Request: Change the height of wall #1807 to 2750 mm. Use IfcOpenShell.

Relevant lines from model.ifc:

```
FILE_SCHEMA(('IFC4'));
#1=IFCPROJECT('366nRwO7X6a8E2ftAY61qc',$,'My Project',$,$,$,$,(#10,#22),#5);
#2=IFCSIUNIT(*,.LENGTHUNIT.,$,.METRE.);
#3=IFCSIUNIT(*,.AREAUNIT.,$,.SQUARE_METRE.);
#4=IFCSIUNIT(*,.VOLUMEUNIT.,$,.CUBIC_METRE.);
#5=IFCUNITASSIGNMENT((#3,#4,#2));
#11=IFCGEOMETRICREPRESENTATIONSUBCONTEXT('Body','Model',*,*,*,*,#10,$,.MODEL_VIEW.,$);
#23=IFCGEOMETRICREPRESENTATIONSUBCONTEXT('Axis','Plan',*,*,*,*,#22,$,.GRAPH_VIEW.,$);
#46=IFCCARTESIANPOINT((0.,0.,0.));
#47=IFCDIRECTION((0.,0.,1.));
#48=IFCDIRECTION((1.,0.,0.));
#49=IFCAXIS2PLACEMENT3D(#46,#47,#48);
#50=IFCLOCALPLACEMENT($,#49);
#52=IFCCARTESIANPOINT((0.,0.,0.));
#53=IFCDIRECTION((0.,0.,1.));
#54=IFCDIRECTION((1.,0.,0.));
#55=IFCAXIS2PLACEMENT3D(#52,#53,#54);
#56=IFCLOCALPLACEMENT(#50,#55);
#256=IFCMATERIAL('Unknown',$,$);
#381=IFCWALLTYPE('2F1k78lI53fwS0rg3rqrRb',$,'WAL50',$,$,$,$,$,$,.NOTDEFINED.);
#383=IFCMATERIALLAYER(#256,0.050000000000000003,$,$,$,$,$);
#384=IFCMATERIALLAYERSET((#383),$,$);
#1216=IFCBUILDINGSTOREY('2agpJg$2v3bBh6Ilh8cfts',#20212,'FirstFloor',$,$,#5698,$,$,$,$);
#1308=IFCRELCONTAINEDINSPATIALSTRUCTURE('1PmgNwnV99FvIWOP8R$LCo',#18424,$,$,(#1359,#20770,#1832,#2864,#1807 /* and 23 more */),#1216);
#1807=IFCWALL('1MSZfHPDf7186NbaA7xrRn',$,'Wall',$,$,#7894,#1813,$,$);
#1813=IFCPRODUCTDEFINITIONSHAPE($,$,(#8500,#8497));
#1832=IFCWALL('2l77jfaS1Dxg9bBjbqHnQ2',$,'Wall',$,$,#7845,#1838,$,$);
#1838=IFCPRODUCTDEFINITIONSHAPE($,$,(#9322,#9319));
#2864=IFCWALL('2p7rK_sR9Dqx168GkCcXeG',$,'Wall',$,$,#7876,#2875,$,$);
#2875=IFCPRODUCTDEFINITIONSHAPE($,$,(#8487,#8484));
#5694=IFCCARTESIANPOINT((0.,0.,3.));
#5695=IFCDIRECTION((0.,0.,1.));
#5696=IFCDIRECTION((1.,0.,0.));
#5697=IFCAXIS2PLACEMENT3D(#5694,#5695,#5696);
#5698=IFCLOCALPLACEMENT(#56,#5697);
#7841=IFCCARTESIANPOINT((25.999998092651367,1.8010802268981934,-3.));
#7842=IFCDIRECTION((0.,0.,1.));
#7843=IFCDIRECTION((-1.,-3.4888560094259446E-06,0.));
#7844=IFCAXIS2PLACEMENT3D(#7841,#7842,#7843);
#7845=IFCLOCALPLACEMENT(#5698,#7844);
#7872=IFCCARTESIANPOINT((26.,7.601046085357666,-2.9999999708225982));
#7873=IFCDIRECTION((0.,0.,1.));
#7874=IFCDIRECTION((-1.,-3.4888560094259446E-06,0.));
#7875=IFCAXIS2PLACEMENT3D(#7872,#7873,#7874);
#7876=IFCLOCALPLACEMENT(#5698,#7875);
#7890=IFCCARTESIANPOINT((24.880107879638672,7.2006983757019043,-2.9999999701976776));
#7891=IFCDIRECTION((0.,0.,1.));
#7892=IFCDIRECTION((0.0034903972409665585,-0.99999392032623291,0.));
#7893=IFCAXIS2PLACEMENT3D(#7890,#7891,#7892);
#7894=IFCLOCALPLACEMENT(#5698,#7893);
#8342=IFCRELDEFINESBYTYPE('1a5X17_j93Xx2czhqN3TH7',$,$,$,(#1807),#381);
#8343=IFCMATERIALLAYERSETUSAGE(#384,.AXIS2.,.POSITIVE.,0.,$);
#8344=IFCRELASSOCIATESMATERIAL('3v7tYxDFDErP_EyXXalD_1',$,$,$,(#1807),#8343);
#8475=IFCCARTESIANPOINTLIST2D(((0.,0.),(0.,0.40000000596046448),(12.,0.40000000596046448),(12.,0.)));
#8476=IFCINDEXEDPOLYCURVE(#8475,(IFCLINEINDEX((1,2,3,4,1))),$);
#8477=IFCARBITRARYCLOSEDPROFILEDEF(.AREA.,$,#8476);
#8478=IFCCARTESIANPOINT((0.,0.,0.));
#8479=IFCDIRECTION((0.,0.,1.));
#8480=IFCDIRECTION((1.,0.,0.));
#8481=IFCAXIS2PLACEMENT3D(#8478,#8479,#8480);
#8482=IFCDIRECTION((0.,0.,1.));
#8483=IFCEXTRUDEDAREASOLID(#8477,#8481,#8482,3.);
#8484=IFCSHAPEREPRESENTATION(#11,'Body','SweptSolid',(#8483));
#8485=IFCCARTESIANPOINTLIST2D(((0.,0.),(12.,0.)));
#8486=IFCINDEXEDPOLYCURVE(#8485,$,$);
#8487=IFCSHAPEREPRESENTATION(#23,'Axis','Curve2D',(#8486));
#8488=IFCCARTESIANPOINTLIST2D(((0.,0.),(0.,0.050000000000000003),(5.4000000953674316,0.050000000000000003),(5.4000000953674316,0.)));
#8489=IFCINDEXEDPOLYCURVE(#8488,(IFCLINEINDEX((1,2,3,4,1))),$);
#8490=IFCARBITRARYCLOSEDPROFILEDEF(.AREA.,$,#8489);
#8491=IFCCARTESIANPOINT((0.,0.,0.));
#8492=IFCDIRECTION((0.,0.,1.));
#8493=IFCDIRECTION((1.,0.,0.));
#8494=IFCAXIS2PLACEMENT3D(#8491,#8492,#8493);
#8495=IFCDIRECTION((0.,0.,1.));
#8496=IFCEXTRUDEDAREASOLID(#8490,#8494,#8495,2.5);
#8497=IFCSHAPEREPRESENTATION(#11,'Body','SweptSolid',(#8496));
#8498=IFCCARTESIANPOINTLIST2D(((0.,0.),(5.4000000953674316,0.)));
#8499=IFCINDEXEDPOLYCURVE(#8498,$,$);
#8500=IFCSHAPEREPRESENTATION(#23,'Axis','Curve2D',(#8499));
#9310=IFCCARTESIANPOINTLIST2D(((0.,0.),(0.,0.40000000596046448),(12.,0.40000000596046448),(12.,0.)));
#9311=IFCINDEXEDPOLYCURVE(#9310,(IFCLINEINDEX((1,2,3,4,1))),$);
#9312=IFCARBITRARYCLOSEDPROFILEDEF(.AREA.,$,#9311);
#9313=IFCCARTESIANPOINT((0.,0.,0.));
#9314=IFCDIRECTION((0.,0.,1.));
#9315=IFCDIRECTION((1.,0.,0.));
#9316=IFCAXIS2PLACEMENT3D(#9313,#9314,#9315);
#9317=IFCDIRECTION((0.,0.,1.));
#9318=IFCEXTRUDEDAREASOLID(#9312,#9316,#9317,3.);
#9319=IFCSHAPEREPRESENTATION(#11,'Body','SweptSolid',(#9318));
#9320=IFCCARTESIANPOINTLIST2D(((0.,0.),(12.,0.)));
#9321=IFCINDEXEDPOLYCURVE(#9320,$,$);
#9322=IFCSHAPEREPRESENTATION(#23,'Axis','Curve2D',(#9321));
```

```python
import ifcopenshell
import ifcopenshell.geom
import ifcopenshell.util.representation
import ifcopenshell.util.shape
import ifcopenshell.util.unit

model = ifcopenshell.open("model.ifc")
unit_scale = ifcopenshell.util.unit.calculate_unit_scale(model)
settings = ifcopenshell.geom.settings()


def volume(element):
    """Net volume in cubic metres, openings subtracted."""
    shape = ifcopenshell.geom.create_shape(settings, element)
    return ifcopenshell.util.shape.get_volume(shape.geometry)


wall = model.by_id(1807)
before = volume(wall)

body = ifcopenshell.util.representation.get_representation(wall, "Model", "Body")
solid = body.Items[0]
old_height = solid.Depth
solid.Depth = 2.75 / unit_scale
after = volume(wall)

print(f"height {old_height:g} -> {solid.Depth:g}, volume {before:.3f} -> {after:.3f} m3")

model.write("model_updated.ifc")
```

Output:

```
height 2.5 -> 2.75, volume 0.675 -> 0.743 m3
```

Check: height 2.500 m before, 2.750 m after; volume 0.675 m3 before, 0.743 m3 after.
